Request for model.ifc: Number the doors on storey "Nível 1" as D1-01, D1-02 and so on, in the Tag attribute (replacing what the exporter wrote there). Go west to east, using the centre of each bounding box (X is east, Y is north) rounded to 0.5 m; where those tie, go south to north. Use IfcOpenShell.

First a look at what the model holds.

```python
import ifcopenshell
import ifcopenshell.util.element
import ifcopenshell.util.placement

model = ifcopenshell.open("model.ifc")
print(model.schema)
storey = next(s for s in model.by_type("IfcBuildingStorey") if s.Name == "Nível 1")
doors = [e for e in ifcopenshell.util.element.get_decomposition(storey) if e.is_a("IfcDoor")]
for e in sorted(doors, key=lambda e: e.id()):
    origin = ifcopenshell.util.placement.get_local_placement(e.ObjectPlacement)[:3, 3]
    print(e.id(), e.Tag, e.Name, origin.round(2) + 0.0, sep=" | ")
```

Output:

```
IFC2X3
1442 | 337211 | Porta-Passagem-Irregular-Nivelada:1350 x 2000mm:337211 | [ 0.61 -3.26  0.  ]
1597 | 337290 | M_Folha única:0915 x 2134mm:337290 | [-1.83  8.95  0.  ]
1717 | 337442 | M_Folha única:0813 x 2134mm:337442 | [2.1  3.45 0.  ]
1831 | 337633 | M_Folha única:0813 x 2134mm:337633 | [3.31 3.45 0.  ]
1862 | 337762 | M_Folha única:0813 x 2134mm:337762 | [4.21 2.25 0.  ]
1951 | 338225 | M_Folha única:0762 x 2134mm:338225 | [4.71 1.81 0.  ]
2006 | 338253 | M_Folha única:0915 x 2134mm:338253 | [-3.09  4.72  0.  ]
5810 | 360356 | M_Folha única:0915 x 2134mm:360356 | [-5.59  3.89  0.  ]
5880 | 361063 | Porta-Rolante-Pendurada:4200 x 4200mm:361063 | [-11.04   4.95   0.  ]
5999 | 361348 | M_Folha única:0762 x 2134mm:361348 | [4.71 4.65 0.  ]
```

```python
import ifcopenshell
import ifcopenshell.geom
import ifcopenshell.util.element
import ifcopenshell.util.shape

model = ifcopenshell.open("model.ifc")
settings = ifcopenshell.geom.settings()
settings.set("use-world-coords", True)


def centre(element):
    shape = ifcopenshell.geom.create_shape(settings, element)
    return ifcopenshell.util.shape.get_bbox_centroid(shape.geometry)


storey = next(s for s in model.by_type("IfcBuildingStorey") if s.Name == "Nível 1")
doors = [e for e in ifcopenshell.util.element.get_decomposition(storey) if e.is_a("IfcDoor")]

# Insertion points can sit at a corner or the storey origin, so sort by the geometry (in metres).
centres = {e: centre(e) for e in doors}
doors.sort(key=lambda e: (round(centres[e][0] / 0.5), centres[e][1]))

for i, e in enumerate(doors, start=1):
    number = f"D1-{i:02d}"
    e.Tag = number
    print(e.id(), number)

model.write("model-out.ifc")
```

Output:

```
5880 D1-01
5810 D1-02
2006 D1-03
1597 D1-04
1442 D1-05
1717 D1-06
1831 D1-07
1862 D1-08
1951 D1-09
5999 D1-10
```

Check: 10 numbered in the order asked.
